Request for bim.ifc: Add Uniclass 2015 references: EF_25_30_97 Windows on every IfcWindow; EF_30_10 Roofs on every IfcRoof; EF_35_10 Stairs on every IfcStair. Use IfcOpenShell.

First a look at what the model holds.

```python
import ifcopenshell

model = ifcopenshell.open("bim.ifc")
print(model.schema)
print("classifications:", [c.Name for c in model.by_type("IfcClassification")])
for ifc_class in ("IfcDoor", "IfcRoof", "IfcStair", "IfcWall", "IfcWindow"):
    print(ifc_class, len(model.by_type(ifc_class)))
```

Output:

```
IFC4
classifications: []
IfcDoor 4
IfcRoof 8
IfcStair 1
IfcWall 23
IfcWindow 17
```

```python
import ifcopenshell
import ifcopenshell.api.classification

model = ifcopenshell.open("bim.ifc")

system = ifcopenshell.api.classification.add_classification(model, classification="Uniclass 2015")

codes = {
    "IfcWindow": ("EF_25_30_97", "Windows"),
    "IfcRoof": ("EF_30_10", "Roofs"),
    "IfcStair": ("EF_35_10", "Stairs"),
}
for ifc_class, (code, name) in codes.items():
    products = model.by_type(ifc_class)
    ifcopenshell.api.classification.add_reference(
        model, products=products, classification=system, identification=code, name=name
    )
    print(code, len(products))

model.write("bim_rev.ifc")
```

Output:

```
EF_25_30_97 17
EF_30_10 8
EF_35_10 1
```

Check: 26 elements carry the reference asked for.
